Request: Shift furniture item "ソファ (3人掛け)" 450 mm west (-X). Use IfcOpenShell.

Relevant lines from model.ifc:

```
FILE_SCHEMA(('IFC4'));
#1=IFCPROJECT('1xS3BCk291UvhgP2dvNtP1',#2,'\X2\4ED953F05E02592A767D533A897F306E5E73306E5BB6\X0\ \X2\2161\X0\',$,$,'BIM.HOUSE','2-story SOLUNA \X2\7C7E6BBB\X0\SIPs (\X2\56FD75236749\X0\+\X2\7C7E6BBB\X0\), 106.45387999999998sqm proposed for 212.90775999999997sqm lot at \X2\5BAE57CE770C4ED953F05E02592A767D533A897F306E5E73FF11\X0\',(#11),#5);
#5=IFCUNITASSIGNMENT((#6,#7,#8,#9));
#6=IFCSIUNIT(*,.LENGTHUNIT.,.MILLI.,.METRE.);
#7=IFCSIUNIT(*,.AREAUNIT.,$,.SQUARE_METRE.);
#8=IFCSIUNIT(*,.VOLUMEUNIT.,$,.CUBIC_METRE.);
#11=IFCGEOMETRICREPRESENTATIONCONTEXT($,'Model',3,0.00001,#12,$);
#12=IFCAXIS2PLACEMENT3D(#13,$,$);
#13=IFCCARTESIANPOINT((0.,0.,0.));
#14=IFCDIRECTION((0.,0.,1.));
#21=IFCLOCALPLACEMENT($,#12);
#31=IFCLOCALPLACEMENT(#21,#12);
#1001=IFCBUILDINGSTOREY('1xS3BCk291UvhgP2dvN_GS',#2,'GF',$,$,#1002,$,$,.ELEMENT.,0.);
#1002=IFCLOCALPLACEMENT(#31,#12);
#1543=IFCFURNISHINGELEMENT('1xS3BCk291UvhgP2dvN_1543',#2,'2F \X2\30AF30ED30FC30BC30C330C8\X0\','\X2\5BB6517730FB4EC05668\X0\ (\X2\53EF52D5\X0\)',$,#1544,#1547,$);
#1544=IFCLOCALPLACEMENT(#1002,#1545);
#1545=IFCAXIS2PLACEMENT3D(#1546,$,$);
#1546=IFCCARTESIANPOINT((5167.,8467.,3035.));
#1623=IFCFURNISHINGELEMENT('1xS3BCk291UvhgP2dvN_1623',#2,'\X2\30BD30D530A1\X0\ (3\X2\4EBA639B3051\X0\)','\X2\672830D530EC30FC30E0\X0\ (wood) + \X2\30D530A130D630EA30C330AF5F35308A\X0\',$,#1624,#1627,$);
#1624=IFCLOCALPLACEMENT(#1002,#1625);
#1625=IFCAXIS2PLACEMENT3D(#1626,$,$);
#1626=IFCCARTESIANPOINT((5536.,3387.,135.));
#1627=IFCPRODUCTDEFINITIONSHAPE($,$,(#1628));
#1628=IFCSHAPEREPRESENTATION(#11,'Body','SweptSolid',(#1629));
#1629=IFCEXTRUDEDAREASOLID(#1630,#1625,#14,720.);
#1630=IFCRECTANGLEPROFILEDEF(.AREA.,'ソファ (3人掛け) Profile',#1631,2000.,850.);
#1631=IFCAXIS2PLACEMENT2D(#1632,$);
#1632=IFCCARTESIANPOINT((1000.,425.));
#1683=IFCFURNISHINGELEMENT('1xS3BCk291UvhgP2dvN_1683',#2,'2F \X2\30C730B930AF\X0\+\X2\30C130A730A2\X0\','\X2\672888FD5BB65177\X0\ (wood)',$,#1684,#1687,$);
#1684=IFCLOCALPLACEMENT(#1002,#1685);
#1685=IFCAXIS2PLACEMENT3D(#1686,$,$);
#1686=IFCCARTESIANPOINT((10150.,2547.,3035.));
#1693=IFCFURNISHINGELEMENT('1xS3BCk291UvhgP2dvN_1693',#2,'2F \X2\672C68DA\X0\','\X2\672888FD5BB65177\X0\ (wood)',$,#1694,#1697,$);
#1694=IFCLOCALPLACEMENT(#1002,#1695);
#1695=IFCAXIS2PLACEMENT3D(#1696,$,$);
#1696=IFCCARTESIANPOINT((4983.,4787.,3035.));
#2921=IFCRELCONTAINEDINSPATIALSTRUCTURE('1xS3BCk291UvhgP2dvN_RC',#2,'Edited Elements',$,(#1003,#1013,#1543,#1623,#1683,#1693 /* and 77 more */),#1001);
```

```python
import ifcopenshell
import ifcopenshell.api.geometry
import ifcopenshell.util.placement
import ifcopenshell.util.unit

model = ifcopenshell.open("model.ifc")
unit_scale = ifcopenshell.util.unit.calculate_unit_scale(model)

item = model.by_guid("1xS3BCk291UvhgP2dvN_1623")
matrix = ifcopenshell.util.placement.get_local_placement(item.ObjectPlacement)
matrix[0, 3] -= 0.45 / unit_scale
ifcopenshell.api.geometry.edit_object_placement(model, product=item, matrix=matrix, is_si=False)

print(ifcopenshell.util.placement.get_local_placement(item.ObjectPlacement).round(3) + 0.0)

model.write("model_updated.ifc")
```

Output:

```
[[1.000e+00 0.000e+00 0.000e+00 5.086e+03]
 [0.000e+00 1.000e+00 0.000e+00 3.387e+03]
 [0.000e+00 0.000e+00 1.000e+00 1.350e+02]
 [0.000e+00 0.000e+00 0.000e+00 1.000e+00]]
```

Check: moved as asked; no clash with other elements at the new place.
